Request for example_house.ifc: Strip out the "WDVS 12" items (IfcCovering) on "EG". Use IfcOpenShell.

First a look at what the model holds.

```python
import ifcopenshell
import ifcopenshell.util.element

model = ifcopenshell.open("example_house.ifc")
print(model.schema)
storey = next(s for s in model.by_type("IfcBuildingStorey") if s.Name == "EG")
coverings = [e for e in ifcopenshell.util.element.get_decomposition(storey) if e.is_a("IfcCovering")]
seen = {}
for e in coverings:
    element_type = ifcopenshell.util.element.get_type(e)
    name = element_type.Name if element_type not in (None, e) else None
    seen[name] = seen.get(name, 0) + 1
for name, count in sorted(seen.items(), key=str):
    print(count, "x", name)
```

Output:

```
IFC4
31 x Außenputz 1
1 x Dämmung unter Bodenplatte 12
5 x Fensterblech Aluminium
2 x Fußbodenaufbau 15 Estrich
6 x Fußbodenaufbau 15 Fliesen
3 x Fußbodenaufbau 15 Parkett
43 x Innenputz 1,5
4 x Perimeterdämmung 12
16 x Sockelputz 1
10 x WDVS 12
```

```python
import ifcopenshell
import ifcopenshell.api.root
import ifcopenshell.util.element

model = ifcopenshell.open("example_house.ifc")

storey = next(s for s in model.by_type("IfcBuildingStorey") if s.Name == "EG")
coverings = [e for e in ifcopenshell.util.element.get_decomposition(storey) if e.is_a("IfcCovering")]
targets = [e for e in coverings if (t := ifcopenshell.util.element.get_type(e)) not in (None, e) and t.Name == "WDVS 12"]

for e in targets:
    ifcopenshell.api.root.remove_product(model, product=e)
print(len(targets), "removed")

model.write("example_house_edited.ifc")
```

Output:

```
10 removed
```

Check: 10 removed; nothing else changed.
